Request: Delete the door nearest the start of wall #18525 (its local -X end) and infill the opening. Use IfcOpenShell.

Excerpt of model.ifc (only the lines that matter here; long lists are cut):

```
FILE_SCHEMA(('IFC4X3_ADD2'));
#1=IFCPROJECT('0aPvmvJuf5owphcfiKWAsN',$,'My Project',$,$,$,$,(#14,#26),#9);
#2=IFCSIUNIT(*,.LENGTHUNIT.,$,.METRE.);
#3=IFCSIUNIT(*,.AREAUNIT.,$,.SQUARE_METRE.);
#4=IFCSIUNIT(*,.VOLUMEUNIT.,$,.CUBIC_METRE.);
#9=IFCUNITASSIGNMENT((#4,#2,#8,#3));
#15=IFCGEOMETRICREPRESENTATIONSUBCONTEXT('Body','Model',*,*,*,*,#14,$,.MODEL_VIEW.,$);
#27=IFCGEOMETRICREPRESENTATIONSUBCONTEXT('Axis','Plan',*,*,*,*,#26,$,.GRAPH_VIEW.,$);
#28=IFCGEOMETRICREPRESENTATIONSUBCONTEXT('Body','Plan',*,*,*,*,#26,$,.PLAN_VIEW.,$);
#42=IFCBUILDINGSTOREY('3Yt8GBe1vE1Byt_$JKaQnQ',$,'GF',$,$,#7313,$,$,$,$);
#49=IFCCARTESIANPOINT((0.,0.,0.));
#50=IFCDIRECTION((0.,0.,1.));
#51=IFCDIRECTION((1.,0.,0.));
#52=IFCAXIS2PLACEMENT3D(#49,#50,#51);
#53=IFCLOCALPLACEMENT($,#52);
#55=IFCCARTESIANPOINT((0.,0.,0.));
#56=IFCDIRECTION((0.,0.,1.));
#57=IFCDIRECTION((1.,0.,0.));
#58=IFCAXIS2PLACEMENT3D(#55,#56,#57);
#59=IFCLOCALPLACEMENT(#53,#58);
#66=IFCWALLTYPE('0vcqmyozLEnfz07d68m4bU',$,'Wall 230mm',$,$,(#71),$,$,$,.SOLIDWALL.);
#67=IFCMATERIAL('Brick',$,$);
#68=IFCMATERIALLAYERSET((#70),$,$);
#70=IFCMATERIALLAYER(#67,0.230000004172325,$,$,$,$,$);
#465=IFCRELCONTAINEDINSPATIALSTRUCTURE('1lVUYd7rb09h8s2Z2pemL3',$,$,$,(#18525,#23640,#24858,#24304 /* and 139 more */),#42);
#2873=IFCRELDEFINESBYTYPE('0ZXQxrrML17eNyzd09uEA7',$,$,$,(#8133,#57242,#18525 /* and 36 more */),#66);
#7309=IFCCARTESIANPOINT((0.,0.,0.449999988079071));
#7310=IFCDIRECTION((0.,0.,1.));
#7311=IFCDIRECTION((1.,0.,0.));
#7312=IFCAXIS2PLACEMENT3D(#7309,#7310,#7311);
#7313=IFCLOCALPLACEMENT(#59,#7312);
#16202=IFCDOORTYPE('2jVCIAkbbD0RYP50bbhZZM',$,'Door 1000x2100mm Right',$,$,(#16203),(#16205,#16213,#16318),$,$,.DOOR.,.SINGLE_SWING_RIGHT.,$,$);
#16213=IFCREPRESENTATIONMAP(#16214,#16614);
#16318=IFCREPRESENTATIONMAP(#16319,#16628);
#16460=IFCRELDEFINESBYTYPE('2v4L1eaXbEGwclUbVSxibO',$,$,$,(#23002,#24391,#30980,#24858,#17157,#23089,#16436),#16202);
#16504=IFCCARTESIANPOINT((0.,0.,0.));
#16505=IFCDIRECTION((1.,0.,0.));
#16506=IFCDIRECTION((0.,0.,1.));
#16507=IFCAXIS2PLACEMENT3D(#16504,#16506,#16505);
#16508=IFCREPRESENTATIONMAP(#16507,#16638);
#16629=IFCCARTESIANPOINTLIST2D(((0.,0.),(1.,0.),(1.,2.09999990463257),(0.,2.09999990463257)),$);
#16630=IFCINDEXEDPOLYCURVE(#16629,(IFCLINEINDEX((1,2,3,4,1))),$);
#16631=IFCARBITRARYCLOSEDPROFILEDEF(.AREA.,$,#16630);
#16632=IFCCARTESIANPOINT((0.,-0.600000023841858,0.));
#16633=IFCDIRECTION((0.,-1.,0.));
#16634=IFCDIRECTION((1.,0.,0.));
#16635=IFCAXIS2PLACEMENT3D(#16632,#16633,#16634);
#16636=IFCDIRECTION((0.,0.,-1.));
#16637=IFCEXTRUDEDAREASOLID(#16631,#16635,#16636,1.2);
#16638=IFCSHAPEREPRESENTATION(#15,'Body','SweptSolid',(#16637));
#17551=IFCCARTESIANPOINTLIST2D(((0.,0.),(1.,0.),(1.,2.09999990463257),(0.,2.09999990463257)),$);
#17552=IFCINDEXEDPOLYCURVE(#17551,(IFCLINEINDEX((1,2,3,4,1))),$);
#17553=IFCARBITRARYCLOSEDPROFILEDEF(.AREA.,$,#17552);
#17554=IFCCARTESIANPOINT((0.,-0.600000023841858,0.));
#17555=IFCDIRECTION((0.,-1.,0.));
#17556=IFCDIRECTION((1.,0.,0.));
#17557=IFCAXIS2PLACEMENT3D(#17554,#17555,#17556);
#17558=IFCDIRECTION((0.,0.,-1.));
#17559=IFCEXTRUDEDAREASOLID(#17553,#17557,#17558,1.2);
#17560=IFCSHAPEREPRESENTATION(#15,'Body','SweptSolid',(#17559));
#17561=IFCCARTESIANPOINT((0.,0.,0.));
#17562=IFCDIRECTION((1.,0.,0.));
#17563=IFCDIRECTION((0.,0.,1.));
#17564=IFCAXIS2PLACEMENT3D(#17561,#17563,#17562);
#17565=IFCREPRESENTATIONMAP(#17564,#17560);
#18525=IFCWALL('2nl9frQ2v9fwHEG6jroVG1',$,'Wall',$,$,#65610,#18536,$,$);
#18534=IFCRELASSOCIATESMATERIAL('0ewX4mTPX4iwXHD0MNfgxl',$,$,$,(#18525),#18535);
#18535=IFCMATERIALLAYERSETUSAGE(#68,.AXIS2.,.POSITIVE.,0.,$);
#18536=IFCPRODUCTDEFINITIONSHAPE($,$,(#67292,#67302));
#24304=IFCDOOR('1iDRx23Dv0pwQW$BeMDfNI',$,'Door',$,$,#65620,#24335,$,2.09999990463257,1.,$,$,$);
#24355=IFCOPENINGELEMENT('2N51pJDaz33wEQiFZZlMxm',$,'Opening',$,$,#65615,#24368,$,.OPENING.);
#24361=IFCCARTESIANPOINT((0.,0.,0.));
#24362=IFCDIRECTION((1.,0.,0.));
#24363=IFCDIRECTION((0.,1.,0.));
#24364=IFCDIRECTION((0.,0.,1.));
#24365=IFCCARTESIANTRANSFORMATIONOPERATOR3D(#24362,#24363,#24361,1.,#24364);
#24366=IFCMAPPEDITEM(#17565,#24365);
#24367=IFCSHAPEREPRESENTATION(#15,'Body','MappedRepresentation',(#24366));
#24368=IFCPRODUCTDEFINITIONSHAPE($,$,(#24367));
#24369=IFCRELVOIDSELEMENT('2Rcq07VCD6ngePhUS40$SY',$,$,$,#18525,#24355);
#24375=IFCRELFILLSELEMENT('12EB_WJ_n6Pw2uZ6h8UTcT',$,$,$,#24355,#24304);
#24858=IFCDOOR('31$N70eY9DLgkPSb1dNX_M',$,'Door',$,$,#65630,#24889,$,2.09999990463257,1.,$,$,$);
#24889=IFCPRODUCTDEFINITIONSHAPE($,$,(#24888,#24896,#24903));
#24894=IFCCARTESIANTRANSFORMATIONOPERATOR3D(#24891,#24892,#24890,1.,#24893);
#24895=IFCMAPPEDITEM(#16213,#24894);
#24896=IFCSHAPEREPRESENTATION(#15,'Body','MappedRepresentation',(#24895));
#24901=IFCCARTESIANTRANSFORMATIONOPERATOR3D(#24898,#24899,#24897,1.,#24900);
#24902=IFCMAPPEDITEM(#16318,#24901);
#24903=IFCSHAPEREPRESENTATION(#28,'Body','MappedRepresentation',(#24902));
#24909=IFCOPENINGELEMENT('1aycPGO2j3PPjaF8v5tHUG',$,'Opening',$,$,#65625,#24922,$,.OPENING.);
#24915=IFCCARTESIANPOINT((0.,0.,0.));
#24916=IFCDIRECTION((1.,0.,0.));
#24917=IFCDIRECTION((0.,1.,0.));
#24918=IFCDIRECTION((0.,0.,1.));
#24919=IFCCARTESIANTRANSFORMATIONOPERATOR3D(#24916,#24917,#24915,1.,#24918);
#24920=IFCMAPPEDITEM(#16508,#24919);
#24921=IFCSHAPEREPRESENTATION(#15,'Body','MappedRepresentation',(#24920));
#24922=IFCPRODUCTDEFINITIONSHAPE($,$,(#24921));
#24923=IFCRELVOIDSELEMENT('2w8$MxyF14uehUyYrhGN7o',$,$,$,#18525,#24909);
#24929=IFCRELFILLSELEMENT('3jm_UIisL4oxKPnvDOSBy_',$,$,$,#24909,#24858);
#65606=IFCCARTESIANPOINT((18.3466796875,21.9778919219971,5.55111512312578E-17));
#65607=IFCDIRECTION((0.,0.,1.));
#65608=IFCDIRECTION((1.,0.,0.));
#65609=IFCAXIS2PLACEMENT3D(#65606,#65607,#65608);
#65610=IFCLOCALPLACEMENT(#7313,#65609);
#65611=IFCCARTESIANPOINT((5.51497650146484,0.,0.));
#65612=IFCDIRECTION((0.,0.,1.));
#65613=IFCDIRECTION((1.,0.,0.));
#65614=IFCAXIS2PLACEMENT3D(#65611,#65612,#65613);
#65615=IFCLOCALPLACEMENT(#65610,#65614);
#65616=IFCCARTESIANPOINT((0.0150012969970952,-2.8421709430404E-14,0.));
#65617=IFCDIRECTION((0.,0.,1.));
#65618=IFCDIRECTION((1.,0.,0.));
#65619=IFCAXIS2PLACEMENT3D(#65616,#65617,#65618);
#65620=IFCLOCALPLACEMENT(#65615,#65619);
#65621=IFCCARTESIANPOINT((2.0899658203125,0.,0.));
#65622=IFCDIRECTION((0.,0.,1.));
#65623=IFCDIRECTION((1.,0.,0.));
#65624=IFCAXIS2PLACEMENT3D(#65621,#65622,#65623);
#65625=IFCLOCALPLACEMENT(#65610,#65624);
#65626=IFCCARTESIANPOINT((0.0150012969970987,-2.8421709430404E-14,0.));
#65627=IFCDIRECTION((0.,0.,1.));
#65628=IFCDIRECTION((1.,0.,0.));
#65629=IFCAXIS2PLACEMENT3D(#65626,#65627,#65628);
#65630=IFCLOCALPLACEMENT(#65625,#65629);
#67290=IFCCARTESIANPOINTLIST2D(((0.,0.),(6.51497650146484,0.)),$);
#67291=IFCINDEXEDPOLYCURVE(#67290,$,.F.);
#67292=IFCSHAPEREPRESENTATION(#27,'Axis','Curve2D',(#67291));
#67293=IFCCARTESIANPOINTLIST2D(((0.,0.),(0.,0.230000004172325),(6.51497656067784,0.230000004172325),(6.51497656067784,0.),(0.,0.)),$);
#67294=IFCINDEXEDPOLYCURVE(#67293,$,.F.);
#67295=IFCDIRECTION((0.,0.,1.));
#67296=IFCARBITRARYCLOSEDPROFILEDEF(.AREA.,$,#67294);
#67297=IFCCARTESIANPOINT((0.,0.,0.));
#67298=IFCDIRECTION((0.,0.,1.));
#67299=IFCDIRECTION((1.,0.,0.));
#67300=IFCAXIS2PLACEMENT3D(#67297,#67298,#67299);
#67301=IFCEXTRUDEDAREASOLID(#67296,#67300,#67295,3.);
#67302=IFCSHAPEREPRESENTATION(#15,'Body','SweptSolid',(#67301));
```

```python
import ifcopenshell
import ifcopenshell.api.feature
import ifcopenshell.api.root
import ifcopenshell.geom
import ifcopenshell.util.shape

model = ifcopenshell.open("model.ifc")
settings = ifcopenshell.geom.settings()


def volume(element):
    """Net volume in cubic metres, openings subtracted."""
    shape = ifcopenshell.geom.create_shape(settings, element)
    return ifcopenshell.util.shape.get_volume(shape.geometry)


door = model.by_id(24858)
opening = door.FillsVoids[0].RelatingOpeningElement
wall = opening.VoidsElements[0].RelatingBuildingElement
before = volume(wall)

ifcopenshell.api.root.remove_product(model, product=door)
ifcopenshell.api.feature.remove_feature(model, feature=opening)

after = volume(wall)

print(f"wall volume {before:.3f} -> {after:.3f} m3")

model.write("model_v2.ifc")
```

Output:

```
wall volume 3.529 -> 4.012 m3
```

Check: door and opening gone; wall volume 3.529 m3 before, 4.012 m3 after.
